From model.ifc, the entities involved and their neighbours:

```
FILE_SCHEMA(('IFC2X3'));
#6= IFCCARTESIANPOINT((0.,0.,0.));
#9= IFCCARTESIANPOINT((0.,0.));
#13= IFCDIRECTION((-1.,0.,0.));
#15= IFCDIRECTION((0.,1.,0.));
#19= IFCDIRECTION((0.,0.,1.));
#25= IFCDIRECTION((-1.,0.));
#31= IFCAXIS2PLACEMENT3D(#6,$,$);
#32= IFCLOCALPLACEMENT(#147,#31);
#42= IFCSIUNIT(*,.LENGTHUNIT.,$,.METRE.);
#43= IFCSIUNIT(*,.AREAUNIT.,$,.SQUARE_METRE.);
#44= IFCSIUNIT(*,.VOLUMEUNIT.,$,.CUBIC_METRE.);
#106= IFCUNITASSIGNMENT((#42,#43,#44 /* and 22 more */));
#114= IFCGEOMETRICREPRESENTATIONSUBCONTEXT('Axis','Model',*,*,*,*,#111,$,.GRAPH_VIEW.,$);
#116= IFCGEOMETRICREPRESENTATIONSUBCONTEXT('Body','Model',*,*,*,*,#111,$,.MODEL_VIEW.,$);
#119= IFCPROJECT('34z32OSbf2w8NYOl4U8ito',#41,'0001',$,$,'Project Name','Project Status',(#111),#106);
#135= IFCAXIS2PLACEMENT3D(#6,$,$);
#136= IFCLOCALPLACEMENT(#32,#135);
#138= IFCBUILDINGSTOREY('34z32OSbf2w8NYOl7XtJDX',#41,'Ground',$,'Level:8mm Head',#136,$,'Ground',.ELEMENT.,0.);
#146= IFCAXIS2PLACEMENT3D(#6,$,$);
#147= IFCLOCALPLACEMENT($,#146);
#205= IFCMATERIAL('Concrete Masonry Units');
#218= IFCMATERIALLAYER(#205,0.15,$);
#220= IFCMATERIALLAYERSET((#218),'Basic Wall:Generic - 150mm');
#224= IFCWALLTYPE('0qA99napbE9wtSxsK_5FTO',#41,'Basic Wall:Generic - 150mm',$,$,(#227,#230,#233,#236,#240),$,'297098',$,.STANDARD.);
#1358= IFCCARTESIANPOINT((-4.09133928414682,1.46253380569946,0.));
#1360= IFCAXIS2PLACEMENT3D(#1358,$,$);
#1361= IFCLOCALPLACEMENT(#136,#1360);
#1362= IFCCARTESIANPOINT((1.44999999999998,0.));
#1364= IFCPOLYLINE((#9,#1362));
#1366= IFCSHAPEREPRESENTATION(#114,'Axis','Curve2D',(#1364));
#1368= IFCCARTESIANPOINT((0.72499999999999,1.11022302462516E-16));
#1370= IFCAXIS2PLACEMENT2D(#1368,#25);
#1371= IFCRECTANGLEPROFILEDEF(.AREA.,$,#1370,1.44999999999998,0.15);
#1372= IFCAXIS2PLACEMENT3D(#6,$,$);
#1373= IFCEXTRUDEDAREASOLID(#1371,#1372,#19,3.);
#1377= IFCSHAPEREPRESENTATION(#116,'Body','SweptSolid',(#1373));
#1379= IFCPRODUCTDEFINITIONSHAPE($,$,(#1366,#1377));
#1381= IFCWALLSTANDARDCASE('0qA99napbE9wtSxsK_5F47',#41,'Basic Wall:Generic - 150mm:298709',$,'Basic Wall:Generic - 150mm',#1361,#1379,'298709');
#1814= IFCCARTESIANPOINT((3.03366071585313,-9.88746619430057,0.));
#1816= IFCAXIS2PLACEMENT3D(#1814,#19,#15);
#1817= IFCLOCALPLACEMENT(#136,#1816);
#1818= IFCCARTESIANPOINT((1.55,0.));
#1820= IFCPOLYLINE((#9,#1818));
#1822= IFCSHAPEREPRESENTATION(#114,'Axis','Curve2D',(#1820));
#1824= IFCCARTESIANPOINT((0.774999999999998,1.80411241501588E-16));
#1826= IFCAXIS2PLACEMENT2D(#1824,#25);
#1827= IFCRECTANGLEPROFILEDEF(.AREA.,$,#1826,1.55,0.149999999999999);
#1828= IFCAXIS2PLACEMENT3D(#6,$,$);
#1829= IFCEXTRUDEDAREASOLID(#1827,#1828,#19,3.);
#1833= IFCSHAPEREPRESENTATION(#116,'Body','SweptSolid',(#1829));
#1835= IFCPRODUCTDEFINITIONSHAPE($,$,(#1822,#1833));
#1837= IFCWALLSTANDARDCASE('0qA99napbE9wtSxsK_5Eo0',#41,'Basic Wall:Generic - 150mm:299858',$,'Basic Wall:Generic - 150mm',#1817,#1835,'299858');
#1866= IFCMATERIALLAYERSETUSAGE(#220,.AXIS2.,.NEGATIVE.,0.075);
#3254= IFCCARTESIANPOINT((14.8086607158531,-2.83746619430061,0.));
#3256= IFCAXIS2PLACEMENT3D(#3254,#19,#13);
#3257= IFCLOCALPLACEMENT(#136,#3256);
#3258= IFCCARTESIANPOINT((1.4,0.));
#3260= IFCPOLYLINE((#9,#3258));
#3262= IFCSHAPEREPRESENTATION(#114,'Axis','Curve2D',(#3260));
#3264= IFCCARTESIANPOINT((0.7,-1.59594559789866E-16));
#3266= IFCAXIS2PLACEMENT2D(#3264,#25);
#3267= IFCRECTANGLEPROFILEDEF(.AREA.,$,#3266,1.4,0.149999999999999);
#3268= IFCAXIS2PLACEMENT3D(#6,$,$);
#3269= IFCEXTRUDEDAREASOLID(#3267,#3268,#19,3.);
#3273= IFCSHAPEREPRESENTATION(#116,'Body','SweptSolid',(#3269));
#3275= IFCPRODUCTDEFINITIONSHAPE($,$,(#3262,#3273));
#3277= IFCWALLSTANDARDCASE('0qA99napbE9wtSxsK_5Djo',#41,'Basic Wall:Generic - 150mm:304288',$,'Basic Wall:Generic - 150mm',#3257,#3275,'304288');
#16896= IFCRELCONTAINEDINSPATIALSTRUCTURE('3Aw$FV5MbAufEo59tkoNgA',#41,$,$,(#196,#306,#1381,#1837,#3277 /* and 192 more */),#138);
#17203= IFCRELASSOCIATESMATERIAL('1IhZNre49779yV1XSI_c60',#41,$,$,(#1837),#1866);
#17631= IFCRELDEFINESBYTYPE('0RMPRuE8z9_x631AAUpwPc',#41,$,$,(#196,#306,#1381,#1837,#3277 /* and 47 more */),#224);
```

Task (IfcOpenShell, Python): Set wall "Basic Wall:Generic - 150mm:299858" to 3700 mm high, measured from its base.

```python
import ifcopenshell
import ifcopenshell.geom
import ifcopenshell.util.representation
import ifcopenshell.util.shape

model = ifcopenshell.open("model.ifc")
settings = ifcopenshell.geom.settings()


def volume(element):
    """Net volume in cubic metres, openings subtracted."""
    shape = ifcopenshell.geom.create_shape(settings, element)
    return ifcopenshell.util.shape.get_volume(shape.geometry)


wall = model.by_guid("0qA99napbE9wtSxsK_5Eo0")
before = volume(wall)

body = ifcopenshell.util.representation.get_representation(wall, "Model", "Body")
solid = body.Items[0]
old_height = solid.Depth
solid.Depth = 3.7
after = volume(wall)

print(f"height {old_height:g} -> {solid.Depth:g}, volume {before:.3f} -> {after:.3f} m3")

model.write("model_edited.ifc")
```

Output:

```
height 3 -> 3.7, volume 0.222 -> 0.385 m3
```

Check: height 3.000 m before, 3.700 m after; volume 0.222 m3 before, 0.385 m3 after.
